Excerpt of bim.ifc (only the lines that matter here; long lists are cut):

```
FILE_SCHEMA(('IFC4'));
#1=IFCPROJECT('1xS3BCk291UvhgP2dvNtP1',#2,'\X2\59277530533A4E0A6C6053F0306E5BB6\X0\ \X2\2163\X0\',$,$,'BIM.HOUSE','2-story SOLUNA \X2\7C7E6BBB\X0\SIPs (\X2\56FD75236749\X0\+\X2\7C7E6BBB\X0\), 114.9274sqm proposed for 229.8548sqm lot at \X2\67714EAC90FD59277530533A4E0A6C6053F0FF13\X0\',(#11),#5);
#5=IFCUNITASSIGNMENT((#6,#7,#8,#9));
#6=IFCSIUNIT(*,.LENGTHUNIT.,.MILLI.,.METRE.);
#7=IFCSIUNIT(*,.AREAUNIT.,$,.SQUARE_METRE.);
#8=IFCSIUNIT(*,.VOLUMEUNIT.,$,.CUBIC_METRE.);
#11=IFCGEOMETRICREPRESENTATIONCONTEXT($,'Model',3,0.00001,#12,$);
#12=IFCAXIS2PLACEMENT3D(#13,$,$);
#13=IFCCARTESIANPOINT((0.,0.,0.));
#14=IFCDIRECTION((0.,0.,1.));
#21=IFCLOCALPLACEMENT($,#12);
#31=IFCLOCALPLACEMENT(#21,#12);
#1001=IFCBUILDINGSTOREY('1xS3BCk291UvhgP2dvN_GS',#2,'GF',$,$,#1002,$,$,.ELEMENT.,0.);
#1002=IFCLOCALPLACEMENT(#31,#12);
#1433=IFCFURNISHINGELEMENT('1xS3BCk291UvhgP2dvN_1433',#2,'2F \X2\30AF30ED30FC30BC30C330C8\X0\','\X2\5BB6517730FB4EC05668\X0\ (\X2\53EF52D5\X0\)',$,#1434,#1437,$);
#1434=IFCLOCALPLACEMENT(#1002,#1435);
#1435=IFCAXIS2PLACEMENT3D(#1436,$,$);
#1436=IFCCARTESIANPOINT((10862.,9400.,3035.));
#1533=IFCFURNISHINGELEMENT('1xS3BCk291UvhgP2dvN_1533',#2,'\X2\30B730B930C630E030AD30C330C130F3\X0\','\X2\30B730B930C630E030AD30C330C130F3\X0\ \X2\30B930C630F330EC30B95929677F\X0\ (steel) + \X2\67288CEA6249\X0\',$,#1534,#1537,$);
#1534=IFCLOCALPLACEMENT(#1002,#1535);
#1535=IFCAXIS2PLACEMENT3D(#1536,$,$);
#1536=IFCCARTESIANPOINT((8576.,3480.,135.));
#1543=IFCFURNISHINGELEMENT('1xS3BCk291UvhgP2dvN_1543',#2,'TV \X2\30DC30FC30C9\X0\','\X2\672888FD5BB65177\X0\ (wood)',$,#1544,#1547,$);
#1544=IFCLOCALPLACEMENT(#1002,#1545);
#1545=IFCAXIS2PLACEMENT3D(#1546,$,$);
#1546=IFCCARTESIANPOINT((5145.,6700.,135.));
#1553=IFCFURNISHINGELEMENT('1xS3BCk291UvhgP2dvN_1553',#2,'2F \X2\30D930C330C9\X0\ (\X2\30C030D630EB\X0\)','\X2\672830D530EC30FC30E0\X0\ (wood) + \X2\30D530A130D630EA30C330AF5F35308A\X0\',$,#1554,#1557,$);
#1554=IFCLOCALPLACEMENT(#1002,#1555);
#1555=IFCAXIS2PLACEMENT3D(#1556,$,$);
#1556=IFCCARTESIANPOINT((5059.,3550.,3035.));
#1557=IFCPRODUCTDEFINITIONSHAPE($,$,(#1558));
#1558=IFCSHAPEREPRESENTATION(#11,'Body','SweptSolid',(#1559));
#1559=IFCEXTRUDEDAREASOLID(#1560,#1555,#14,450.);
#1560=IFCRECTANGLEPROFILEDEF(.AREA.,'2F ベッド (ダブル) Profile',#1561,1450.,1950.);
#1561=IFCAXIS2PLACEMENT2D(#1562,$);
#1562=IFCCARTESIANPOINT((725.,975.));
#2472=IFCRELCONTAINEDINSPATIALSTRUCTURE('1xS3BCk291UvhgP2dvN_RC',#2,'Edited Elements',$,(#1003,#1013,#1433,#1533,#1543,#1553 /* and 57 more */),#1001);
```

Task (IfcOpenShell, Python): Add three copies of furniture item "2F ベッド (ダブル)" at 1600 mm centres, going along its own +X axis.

```python
import ifcopenshell
import ifcopenshell.api.geometry
import ifcopenshell.api.root
import ifcopenshell.util.element
import ifcopenshell.util.placement
import ifcopenshell.util.unit

model = ifcopenshell.open("bim.ifc")
unit_scale = ifcopenshell.util.unit.calculate_unit_scale(model)


def reuse_history(source, copy):
    """copy_class also copies each property set's owner history, people and application; keep the originals."""
    for rel in copy.IsDefinedBy:
        if rel.is_a("IfcRelDefinesByProperties") and (history := rel.RelatingPropertyDefinition.OwnerHistory):
            rel.RelatingPropertyDefinition.OwnerHistory = source.OwnerHistory
            ifcopenshell.util.element.remove_deep2(model, history)


source = model.by_id(1553)
base = ifcopenshell.util.placement.get_local_placement(source.ObjectPlacement)
step = base[:3, 0] * 1.6 / unit_scale

for i in range(1, 4):
    copy = ifcopenshell.api.root.copy_class(model, product=source)
    copy.Representation = ifcopenshell.util.element.copy_deep(
        model, source.Representation, exclude=["IfcGeometricRepresentationContext", "IfcRepresentationMap"]
    )
    reuse_history(source, copy)
    matrix = base.copy()
    matrix[:3, 3] += i * step
    print("added at", matrix[:3, 3].round(3) + 0.0)
    ifcopenshell.api.geometry.edit_object_placement(model, product=copy, matrix=matrix, is_si=False)

model.write("bim-out.ifc")
```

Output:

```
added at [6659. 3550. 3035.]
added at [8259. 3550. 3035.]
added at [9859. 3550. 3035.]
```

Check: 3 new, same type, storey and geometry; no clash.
